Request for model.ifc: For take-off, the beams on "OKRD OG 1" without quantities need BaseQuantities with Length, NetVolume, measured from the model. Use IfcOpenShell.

First a look at what the model holds.

```python
import ifcopenshell
import ifcopenshell.util.element
import ifcopenshell.util.unit

model = ifcopenshell.open("model.ifc")
print(model.schema)
for unit_type in ("LENGTHUNIT", "AREAUNIT", "VOLUMEUNIT"):
    print(unit_type, ifcopenshell.util.unit.calculate_unit_scale(model, unit_type))
storey = next(s for s in model.by_type("IfcBuildingStorey") if s.Name == "OKRD OG 1")
beams = [e for e in ifcopenshell.util.element.get_decomposition(storey) if e.is_a("IfcBeam")]
for e in sorted(beams, key=lambda e: e.id()):
    print(e.id(), e.is_a(), e.Name, list(ifcopenshell.util.element.get_psets(e, qtos_only=True)), sep=" | ")
```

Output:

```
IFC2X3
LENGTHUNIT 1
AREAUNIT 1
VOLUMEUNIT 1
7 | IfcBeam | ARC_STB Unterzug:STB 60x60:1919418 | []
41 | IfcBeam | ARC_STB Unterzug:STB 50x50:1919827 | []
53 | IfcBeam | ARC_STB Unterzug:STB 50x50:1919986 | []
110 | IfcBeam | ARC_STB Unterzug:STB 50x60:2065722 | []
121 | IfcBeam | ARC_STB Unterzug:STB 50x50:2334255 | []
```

```python
import ifcopenshell
import ifcopenshell.api.pset
import ifcopenshell.geom
import ifcopenshell.util.element
import ifcopenshell.util.shape
import ifcopenshell.util.unit

model = ifcopenshell.open("model.ifc")
unit_scale = ifcopenshell.util.unit.calculate_unit_scale(model)
volume_scale = ifcopenshell.util.unit.calculate_unit_scale(model, "VOLUMEUNIT")
settings = ifcopenshell.geom.settings()

storey = next(s for s in model.by_type("IfcBuildingStorey") if s.Name == "OKRD OG 1")
beams = [e for e in ifcopenshell.util.element.get_decomposition(storey) if e.is_a("IfcBeam")]

for e in sorted(beams, key=lambda e: e.id()):
    if ifcopenshell.util.element.get_psets(e, qtos_only=True, should_inherit=False):
        continue
    # Geometry comes back in metres, in the element's own axes.
    shape = ifcopenshell.geom.create_shape(settings, e)
    values = {
        "Length": ifcopenshell.util.shape.get_max_xyz(shape.geometry) / unit_scale,
        "NetVolume": ifcopenshell.util.shape.get_volume(shape.geometry) / volume_scale,
    }
    qto = ifcopenshell.api.pset.add_qto(model, product=e, name="BaseQuantities")
    ifcopenshell.api.pset.edit_qto(model, qto=qto, properties=values)
    print(e.id(), {k: round(v, 3) for k, v in values.items()})

model.write("model_rev.ifc")
```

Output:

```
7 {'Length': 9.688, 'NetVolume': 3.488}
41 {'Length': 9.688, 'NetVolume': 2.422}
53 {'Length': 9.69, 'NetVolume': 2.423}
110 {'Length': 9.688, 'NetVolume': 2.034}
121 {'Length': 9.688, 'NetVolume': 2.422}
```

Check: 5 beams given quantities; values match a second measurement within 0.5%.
